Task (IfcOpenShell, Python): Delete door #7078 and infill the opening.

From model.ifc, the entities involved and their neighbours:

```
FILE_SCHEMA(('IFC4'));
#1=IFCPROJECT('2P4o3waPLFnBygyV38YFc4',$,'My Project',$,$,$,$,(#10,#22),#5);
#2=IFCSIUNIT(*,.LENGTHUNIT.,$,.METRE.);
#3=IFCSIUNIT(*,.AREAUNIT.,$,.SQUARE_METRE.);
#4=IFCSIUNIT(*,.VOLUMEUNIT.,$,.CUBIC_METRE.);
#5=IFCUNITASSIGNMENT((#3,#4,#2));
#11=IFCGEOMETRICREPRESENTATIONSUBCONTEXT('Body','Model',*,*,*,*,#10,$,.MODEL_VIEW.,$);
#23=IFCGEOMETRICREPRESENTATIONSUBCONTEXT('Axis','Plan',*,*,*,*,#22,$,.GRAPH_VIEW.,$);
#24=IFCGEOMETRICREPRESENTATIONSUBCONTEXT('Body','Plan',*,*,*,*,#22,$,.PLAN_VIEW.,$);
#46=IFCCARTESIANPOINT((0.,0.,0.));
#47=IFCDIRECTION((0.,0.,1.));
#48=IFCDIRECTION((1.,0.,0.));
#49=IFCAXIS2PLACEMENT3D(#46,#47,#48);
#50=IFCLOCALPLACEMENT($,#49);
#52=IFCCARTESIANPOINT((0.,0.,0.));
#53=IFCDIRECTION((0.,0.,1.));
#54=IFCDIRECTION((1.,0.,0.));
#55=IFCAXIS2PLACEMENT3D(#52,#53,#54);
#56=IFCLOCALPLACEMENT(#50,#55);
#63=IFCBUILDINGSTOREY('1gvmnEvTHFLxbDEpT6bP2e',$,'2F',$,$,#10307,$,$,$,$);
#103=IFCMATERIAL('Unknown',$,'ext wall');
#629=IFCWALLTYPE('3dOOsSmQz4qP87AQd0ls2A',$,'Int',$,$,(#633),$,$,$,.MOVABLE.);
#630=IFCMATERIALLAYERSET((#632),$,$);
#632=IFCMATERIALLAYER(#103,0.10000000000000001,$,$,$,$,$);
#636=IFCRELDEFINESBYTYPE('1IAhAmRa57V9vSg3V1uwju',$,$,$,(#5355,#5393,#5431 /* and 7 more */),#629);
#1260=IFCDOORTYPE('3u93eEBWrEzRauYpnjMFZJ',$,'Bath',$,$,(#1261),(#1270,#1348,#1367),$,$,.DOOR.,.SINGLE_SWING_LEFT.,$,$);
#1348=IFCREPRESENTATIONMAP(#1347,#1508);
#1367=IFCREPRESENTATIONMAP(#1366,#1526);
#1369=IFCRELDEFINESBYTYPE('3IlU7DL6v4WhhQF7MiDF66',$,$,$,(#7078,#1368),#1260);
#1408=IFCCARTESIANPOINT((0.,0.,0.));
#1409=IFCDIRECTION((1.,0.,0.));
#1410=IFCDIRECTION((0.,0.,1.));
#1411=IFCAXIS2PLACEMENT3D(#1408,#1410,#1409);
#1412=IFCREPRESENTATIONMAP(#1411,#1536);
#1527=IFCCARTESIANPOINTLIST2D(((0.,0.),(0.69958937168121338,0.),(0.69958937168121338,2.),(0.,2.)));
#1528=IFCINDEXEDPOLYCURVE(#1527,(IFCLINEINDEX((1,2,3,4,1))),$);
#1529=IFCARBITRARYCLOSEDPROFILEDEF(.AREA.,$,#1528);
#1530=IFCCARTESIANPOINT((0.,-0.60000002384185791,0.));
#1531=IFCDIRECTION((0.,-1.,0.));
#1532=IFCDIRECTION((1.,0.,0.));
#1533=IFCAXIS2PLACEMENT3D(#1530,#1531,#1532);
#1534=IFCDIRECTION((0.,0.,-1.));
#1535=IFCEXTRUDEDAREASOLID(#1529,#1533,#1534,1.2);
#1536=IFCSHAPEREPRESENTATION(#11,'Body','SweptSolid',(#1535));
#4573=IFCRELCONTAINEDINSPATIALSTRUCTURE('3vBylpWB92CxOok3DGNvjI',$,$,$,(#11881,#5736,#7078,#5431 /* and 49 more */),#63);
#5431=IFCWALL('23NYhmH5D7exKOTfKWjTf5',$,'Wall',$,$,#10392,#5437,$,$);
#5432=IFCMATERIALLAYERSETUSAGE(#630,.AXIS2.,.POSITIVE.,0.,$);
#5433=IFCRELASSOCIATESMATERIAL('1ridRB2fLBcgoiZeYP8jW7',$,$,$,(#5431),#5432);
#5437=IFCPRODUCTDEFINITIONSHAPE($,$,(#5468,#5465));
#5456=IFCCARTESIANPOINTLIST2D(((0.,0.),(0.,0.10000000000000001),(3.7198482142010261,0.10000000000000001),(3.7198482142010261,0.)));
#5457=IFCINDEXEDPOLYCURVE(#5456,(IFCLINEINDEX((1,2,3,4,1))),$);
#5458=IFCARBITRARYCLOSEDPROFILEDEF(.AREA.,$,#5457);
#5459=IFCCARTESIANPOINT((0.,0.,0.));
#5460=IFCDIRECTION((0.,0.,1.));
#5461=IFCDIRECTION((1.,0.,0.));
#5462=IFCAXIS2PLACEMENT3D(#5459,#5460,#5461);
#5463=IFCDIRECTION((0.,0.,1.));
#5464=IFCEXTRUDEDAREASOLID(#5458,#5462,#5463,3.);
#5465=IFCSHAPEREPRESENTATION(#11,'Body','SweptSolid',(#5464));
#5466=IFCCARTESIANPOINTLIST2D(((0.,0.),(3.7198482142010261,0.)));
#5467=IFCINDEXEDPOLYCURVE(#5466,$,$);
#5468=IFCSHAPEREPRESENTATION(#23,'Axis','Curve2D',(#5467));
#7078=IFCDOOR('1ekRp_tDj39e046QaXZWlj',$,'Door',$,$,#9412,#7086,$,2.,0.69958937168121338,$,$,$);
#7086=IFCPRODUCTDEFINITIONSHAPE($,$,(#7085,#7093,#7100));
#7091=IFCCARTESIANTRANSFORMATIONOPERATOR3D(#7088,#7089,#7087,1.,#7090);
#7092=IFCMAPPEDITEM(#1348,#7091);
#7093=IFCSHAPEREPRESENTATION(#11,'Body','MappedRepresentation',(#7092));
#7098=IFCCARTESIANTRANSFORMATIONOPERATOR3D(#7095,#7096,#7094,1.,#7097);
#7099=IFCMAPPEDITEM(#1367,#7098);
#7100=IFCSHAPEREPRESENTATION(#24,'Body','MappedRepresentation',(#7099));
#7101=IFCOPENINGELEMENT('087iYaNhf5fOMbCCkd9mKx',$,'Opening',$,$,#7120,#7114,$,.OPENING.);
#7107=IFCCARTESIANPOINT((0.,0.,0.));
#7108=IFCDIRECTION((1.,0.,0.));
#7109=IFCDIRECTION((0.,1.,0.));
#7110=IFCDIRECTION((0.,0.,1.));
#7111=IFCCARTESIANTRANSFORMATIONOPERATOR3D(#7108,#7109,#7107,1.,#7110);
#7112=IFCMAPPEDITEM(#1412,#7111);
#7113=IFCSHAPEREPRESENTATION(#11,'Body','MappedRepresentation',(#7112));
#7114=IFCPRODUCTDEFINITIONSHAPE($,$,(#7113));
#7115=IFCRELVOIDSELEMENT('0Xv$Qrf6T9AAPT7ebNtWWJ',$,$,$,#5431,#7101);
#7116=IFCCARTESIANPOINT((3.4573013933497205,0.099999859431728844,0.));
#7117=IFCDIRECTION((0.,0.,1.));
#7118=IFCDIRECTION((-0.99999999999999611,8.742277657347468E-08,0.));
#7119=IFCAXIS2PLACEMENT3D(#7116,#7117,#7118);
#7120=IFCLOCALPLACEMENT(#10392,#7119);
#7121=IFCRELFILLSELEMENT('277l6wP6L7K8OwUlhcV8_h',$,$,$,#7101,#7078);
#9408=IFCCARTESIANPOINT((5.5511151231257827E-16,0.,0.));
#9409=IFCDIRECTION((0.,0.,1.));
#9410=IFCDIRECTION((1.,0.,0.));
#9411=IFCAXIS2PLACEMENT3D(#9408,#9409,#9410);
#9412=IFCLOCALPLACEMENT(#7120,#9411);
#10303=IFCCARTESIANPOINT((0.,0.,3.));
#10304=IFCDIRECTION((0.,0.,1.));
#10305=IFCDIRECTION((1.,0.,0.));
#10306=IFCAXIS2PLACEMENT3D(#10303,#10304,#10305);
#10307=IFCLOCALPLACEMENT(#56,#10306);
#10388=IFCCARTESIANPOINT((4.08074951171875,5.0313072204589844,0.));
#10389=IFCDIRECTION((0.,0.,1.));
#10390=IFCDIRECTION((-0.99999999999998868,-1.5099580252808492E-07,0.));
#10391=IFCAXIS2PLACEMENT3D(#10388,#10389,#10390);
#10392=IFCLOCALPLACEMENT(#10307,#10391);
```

```python
import ifcopenshell
import ifcopenshell.api.feature
import ifcopenshell.api.root
import ifcopenshell.geom
import ifcopenshell.util.shape

model = ifcopenshell.open("model.ifc")
settings = ifcopenshell.geom.settings()


def volume(element):
    """Net volume in cubic metres, openings subtracted."""
    shape = ifcopenshell.geom.create_shape(settings, element)
    return ifcopenshell.util.shape.get_volume(shape.geometry)


door = model.by_guid("1ekRp_tDj39e046QaXZWlj")
opening = door.FillsVoids[0].RelatingOpeningElement
wall = opening.VoidsElements[0].RelatingBuildingElement
before = volume(wall)

ifcopenshell.api.root.remove_product(model, product=door)
ifcopenshell.api.feature.remove_feature(model, feature=opening)

after = volume(wall)

print(f"wall volume {before:.3f} -> {after:.3f} m3")

model.write("model_v2.ifc")
```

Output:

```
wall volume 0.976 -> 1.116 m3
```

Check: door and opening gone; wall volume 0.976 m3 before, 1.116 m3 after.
